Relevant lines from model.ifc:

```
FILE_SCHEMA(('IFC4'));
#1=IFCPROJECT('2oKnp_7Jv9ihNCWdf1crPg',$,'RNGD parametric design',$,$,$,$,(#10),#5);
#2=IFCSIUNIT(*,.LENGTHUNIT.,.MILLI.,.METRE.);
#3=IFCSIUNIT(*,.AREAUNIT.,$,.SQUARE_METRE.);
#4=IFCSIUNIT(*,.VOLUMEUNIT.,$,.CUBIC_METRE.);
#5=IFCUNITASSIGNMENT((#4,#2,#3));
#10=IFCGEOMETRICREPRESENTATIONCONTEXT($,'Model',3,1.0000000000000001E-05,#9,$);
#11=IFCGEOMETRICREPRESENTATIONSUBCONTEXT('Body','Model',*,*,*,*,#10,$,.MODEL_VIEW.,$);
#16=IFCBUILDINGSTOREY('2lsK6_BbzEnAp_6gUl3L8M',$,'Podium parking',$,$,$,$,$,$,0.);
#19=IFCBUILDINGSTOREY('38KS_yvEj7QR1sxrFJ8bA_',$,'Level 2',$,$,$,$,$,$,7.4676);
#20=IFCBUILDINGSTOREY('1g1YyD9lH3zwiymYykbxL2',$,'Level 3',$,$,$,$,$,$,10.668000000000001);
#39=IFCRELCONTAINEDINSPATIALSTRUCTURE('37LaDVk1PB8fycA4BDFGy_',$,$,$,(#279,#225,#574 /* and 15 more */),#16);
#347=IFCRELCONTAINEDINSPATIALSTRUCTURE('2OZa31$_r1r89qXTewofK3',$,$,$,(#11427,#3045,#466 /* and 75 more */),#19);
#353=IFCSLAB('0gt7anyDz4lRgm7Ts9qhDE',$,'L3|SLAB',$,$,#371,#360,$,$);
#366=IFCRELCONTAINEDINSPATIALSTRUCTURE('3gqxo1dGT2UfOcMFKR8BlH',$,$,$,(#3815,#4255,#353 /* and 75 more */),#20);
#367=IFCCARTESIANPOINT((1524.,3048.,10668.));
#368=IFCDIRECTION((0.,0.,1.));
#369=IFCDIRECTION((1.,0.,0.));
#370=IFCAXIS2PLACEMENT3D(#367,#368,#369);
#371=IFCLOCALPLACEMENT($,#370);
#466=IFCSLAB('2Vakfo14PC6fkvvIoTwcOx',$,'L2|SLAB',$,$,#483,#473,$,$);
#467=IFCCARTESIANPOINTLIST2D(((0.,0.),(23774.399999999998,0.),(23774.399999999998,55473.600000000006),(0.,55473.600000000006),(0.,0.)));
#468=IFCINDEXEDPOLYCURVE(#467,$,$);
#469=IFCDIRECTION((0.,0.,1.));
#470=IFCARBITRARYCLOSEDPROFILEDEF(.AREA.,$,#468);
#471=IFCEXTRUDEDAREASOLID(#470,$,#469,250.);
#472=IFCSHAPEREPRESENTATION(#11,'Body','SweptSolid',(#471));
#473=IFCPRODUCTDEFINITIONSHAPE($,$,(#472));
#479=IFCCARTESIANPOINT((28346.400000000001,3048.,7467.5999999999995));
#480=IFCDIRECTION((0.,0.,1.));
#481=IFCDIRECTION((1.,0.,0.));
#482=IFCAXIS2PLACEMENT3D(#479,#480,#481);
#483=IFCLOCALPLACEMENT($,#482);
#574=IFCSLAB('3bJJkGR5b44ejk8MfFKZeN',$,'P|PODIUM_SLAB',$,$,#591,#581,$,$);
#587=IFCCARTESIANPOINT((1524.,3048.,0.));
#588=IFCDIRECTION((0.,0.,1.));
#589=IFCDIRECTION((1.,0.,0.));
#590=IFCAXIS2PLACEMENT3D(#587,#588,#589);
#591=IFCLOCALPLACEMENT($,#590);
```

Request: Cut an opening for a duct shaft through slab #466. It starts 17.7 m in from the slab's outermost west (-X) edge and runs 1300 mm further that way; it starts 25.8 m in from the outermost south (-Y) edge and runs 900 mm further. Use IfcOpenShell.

```python
import numpy as np
import ifcopenshell
import ifcopenshell.api.feature
import ifcopenshell.api.geometry
import ifcopenshell.api.root
import ifcopenshell.geom
import ifcopenshell.util.placement
import ifcopenshell.util.representation
import ifcopenshell.util.shape
import ifcopenshell.util.unit

model = ifcopenshell.open("model.ifc")
unit_scale = ifcopenshell.util.unit.calculate_unit_scale(model)
settings = ifcopenshell.geom.settings()


def volume(element):
    """Net volume in cubic metres, openings subtracted."""
    shape = ifcopenshell.geom.create_shape(settings, element)
    return ifcopenshell.util.shape.get_volume(shape.geometry)


slab = model.by_id(466)
before = volume(slab)

# Extent in the slab's own axes, in metres. The edges named are its -X and -Y sides.
slab_shape = ifcopenshell.geom.create_shape(settings, slab)
vertices = ifcopenshell.util.shape.get_vertices(slab_shape.geometry)
x_min, y_min, bottom = vertices.min(axis=0)
top = vertices[:, 2].max()

opening = ifcopenshell.api.root.create_entity(model, ifc_class="IfcOpeningElement", name="Duct shaft opening", predefined_type="OPENING")
context = ifcopenshell.util.representation.get_context(model, "Model", "Body", "MODEL_VIEW")
width, depth = 1.3, 0.9
outline = [(0.0, 0.0), (width, 0.0), (width, depth), (0.0, depth), (0.0, 0.0)]
# Overshoot both faces by 50 mm so the cut is clean.
shape = ifcopenshell.api.geometry.add_slab_representation(
    model, context=context, depth=top - bottom + 0.1, polyline=outline
)
ifcopenshell.api.geometry.assign_representation(model, product=opening, representation=shape)

matrix = ifcopenshell.util.placement.get_local_placement(slab.ObjectPlacement)
matrix[:, 3] = matrix @ np.append(np.array([x_min + 17.7, y_min + 25.8, bottom - 0.05]) / unit_scale, 1.0)
ifcopenshell.api.geometry.edit_object_placement(model, product=opening, matrix=matrix, is_si=False)
ifcopenshell.api.feature.add_feature(model, feature=opening, element=slab)

after = volume(slab)

print(f"slab volume {before:.3f} -> {after:.3f} m3")

model.write("model_updated.ifc")
```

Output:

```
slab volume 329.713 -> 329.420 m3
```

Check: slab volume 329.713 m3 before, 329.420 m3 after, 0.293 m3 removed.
